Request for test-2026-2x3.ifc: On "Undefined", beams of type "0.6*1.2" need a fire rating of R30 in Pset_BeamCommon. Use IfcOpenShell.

First a look at what the model holds.

```python
import ifcopenshell
import ifcopenshell.util.element

model = ifcopenshell.open("test-2026-2x3.ifc")
print(model.schema)
storey = next(s for s in model.by_type("IfcBuildingStorey") if s.Name == "Undefined")
beams = [e for e in ifcopenshell.util.element.get_decomposition(storey) if e.is_a("IfcBeam")]
seen = {}
for e in beams:
    element_type = ifcopenshell.util.element.get_type(e)
    key = (element_type.Name if element_type != e and element_type else None, ifcopenshell.util.element.get_pset(e, "Pset_BeamCommon", "FireRating"))
    seen[key] = seen.get(key, 0) + 1
for (name, value), count in sorted(seen.items(), key=str):
    print(count, "x", name, "|", value)
```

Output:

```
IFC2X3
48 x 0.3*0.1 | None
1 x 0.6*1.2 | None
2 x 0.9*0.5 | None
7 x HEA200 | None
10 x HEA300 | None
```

```python
import ifcopenshell
import ifcopenshell.api.pset
import ifcopenshell.util.element

model = ifcopenshell.open("test-2026-2x3.ifc")

storey = next(s for s in model.by_type("IfcBuildingStorey") if s.Name == "Undefined")
beams = [e for e in ifcopenshell.util.element.get_decomposition(storey) if e.is_a("IfcBeam")]

count = 0
for e in beams:
    element_type = ifcopenshell.util.element.get_type(e)
    if element_type in (None, e) or element_type.Name != "0.6*1.2":
        continue
    # add_pset returns the element's existing set when there is one.
    pset = ifcopenshell.api.pset.add_pset(model, product=e, name="Pset_BeamCommon")
    ifcopenshell.api.pset.edit_pset(model, pset=pset, properties={"FireRating": "R30"})
    count += 1

print(count, "beams updated")

model.write("test-2026-2x3_edited.ifc")
```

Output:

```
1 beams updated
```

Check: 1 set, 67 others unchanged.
